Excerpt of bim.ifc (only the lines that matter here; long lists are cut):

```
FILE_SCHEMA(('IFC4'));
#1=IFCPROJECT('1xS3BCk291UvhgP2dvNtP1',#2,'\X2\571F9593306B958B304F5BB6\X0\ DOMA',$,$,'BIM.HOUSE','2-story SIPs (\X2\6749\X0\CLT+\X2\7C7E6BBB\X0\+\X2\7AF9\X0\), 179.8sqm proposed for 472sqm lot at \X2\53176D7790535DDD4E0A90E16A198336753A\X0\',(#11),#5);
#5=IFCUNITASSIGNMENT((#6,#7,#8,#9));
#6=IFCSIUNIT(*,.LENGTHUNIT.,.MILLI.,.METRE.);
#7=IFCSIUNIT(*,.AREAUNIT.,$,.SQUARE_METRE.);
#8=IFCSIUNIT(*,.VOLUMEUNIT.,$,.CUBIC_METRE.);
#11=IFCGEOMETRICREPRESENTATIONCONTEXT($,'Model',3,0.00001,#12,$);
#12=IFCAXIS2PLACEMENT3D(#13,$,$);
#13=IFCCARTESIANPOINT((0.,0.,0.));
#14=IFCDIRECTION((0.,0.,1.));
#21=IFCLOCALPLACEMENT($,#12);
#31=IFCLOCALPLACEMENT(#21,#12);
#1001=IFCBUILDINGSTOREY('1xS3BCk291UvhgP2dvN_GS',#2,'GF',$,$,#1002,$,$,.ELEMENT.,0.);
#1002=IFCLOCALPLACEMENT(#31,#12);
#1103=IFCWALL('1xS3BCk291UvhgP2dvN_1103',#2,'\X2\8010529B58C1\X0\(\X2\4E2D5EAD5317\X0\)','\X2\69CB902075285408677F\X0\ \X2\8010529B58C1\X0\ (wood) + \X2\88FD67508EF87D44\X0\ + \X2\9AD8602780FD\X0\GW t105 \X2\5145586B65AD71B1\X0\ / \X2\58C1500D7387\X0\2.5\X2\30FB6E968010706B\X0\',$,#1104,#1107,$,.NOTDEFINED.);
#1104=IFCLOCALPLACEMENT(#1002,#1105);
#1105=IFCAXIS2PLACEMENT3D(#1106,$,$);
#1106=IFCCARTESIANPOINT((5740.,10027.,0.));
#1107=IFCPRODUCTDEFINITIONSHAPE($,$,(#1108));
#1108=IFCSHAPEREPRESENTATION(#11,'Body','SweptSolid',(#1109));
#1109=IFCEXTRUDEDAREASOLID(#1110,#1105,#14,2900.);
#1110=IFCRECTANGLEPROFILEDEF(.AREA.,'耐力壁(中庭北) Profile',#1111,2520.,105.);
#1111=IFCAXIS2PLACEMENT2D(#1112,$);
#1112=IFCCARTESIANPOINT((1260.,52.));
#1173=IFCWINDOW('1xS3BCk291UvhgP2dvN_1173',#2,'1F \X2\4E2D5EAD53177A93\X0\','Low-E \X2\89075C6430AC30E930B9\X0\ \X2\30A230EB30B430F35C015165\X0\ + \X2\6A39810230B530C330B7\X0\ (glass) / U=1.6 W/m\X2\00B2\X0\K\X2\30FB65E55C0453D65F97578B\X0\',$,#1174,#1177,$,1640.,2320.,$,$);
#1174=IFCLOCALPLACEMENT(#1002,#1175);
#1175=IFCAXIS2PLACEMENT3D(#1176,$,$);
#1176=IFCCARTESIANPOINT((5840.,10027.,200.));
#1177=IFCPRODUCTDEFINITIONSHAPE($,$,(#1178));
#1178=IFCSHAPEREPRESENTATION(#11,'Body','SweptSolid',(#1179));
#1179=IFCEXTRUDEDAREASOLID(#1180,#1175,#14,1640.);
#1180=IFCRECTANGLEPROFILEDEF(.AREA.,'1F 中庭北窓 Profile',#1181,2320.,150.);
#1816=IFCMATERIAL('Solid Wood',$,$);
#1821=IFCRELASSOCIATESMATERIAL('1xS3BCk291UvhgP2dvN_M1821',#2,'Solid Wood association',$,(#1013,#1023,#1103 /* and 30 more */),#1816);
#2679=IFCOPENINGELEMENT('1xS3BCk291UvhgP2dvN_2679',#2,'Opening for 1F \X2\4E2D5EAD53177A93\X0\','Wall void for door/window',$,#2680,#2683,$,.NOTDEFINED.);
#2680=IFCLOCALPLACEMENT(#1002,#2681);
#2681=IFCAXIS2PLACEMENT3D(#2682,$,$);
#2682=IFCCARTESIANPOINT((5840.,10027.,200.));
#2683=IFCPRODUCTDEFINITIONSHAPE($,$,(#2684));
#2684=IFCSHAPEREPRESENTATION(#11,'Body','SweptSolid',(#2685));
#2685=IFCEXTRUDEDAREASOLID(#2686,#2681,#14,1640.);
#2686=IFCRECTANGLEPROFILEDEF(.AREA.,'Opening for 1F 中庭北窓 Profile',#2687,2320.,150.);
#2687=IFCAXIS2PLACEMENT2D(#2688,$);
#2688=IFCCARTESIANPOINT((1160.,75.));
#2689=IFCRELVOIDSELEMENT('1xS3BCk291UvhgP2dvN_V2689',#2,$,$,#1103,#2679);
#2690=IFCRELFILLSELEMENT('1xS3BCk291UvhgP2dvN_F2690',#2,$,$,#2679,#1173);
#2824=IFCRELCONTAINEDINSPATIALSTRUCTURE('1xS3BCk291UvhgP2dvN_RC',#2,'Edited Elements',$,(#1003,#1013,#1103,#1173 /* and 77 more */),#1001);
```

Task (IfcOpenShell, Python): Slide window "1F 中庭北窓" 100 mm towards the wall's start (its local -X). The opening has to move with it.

```python
import ifcopenshell
import ifcopenshell.api.geometry
import ifcopenshell.util.placement
import ifcopenshell.util.unit

model = ifcopenshell.open("bim.ifc")
unit_scale = ifcopenshell.util.unit.calculate_unit_scale(model)

window = model.by_guid("1xS3BCk291UvhgP2dvN_1173")
opening = window.FillsVoids[0].RelatingOpeningElement
wall = opening.VoidsElements[0].RelatingBuildingElement

wall_matrix = ifcopenshell.util.placement.get_local_placement(wall.ObjectPlacement)
shift = wall_matrix[:3, 0] * -0.1 / unit_scale
before = ifcopenshell.util.placement.get_local_placement(window.ObjectPlacement)[:3, 3].copy()

# The window is not placed relative to its opening, so move both.
for product in (opening, window):
    matrix = ifcopenshell.util.placement.get_local_placement(product.ObjectPlacement)
    matrix[:3, 3] += shift
    ifcopenshell.api.geometry.edit_object_placement(model, product=product, matrix=matrix, is_si=False)

after = ifcopenshell.util.placement.get_local_placement(window.ObjectPlacement)[:3, 3]
print("window moved by", (after - before).round(3) + 0.0)

model.write("bim_v2.ifc")
```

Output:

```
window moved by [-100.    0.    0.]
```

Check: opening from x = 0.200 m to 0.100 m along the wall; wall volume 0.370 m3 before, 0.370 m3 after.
